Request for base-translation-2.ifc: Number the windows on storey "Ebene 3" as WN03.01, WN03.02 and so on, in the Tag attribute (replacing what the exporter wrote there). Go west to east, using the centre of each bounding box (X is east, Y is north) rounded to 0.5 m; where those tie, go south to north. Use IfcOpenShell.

First a look at what the model holds.

```python
import ifcopenshell
import ifcopenshell.util.element
import ifcopenshell.util.placement

model = ifcopenshell.open("base-translation-2.ifc")
print(model.schema)
storey = next(s for s in model.by_type("IfcBuildingStorey") if s.Name == "Ebene 3")
windows = [e for e in ifcopenshell.util.element.get_decomposition(storey) if e.is_a("IfcWindow")]
for e in sorted(windows, key=lambda e: e.id()):
    origin = ifcopenshell.util.placement.get_local_placement(e.ObjectPlacement)[:3, 3]
    print(e.id(), e.Tag, e.Name, origin.round(2) + 0.0, sep=" | ")
```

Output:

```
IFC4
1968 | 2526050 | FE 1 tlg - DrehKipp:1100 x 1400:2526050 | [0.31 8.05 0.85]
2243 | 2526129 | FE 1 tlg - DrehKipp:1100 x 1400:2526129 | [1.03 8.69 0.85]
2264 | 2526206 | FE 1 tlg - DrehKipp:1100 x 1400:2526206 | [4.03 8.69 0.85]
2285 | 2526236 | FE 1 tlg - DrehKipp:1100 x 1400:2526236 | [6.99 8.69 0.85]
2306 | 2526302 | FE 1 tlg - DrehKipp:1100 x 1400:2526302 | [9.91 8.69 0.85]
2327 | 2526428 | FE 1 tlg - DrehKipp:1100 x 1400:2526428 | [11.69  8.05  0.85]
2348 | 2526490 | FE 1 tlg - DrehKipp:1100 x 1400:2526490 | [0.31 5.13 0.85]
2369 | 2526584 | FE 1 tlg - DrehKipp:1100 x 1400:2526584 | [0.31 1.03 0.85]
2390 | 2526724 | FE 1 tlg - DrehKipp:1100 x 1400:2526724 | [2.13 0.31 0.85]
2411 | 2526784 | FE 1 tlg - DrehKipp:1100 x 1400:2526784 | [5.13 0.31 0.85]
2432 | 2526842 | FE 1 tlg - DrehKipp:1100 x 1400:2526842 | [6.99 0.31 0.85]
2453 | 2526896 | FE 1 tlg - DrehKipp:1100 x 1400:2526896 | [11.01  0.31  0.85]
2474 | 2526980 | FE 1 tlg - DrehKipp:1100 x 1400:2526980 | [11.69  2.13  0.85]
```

```python
import ifcopenshell
import ifcopenshell.geom
import ifcopenshell.util.element
import ifcopenshell.util.shape

model = ifcopenshell.open("base-translation-2.ifc")
settings = ifcopenshell.geom.settings()
settings.set("use-world-coords", True)


def centre(element):
    shape = ifcopenshell.geom.create_shape(settings, element)
    return ifcopenshell.util.shape.get_bbox_centroid(shape.geometry)


storey = next(s for s in model.by_type("IfcBuildingStorey") if s.Name == "Ebene 3")
windows = [e for e in ifcopenshell.util.element.get_decomposition(storey) if e.is_a("IfcWindow")]

# Insertion points can sit at a corner or the storey origin, so sort by the geometry (in metres).
centres = {e: centre(e) for e in windows}
windows.sort(key=lambda e: (round(centres[e][0] / 0.5), centres[e][1]))

for i, e in enumerate(windows, start=1):
    number = f"WN03.{i:02d}"
    e.Tag = number
    print(e.id(), number)

model.write("base-translation-2_edited.ifc")
```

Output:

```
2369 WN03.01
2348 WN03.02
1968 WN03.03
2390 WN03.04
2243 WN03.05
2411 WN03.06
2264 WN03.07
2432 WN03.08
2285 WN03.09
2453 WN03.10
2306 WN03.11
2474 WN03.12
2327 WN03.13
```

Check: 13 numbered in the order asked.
